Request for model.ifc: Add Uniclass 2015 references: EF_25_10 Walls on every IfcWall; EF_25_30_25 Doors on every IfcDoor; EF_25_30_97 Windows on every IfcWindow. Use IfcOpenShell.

First a look at what the model holds.

```python
import ifcopenshell

model = ifcopenshell.open("model.ifc")
print(model.schema)
print("classifications:", [c.Name for c in model.by_type("IfcClassification")])
for ifc_class in ("IfcDoor", "IfcRoof", "IfcStair", "IfcWall", "IfcWindow"):
    print(ifc_class, len(model.by_type(ifc_class)))
```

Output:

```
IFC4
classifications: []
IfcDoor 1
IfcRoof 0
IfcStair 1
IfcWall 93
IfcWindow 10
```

```python
import ifcopenshell
import ifcopenshell.api.classification

model = ifcopenshell.open("model.ifc")

system = ifcopenshell.api.classification.add_classification(model, classification="Uniclass 2015")

codes = {
    "IfcWall": ("EF_25_10", "Walls"),
    "IfcDoor": ("EF_25_30_25", "Doors"),
    "IfcWindow": ("EF_25_30_97", "Windows"),
}
for ifc_class, (code, name) in codes.items():
    products = model.by_type(ifc_class)
    ifcopenshell.api.classification.add_reference(
        model, products=products, classification=system, identification=code, name=name
    )
    print(code, len(products))

model.write("model_edited.ifc")
```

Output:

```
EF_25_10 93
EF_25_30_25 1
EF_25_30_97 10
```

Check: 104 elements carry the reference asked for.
